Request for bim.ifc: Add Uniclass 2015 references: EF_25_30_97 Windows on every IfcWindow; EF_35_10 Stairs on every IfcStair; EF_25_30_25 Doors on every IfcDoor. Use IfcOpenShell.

First a look at what the model holds.

```python
import ifcopenshell

model = ifcopenshell.open("bim.ifc")
print(model.schema)
print("classifications:", [c.Name for c in model.by_type("IfcClassification")])
for ifc_class in ("IfcDoor", "IfcRoof", "IfcStair", "IfcWall", "IfcWindow"):
    print(ifc_class, len(model.by_type(ifc_class)))
```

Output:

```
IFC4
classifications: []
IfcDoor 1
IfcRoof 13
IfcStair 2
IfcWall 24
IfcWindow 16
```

```python
import ifcopenshell
import ifcopenshell.api.classification

model = ifcopenshell.open("bim.ifc")

system = ifcopenshell.api.classification.add_classification(model, classification="Uniclass 2015")

codes = {
    "IfcWindow": ("EF_25_30_97", "Windows"),
    "IfcStair": ("EF_35_10", "Stairs"),
    "IfcDoor": ("EF_25_30_25", "Doors"),
}
for ifc_class, (code, name) in codes.items():
    products = model.by_type(ifc_class)
    ifcopenshell.api.classification.add_reference(
        model, products=products, classification=system, identification=code, name=name
    )
    print(code, len(products))

model.write("bim_edited.ifc")
```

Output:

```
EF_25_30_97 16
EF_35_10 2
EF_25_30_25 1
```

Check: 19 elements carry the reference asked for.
